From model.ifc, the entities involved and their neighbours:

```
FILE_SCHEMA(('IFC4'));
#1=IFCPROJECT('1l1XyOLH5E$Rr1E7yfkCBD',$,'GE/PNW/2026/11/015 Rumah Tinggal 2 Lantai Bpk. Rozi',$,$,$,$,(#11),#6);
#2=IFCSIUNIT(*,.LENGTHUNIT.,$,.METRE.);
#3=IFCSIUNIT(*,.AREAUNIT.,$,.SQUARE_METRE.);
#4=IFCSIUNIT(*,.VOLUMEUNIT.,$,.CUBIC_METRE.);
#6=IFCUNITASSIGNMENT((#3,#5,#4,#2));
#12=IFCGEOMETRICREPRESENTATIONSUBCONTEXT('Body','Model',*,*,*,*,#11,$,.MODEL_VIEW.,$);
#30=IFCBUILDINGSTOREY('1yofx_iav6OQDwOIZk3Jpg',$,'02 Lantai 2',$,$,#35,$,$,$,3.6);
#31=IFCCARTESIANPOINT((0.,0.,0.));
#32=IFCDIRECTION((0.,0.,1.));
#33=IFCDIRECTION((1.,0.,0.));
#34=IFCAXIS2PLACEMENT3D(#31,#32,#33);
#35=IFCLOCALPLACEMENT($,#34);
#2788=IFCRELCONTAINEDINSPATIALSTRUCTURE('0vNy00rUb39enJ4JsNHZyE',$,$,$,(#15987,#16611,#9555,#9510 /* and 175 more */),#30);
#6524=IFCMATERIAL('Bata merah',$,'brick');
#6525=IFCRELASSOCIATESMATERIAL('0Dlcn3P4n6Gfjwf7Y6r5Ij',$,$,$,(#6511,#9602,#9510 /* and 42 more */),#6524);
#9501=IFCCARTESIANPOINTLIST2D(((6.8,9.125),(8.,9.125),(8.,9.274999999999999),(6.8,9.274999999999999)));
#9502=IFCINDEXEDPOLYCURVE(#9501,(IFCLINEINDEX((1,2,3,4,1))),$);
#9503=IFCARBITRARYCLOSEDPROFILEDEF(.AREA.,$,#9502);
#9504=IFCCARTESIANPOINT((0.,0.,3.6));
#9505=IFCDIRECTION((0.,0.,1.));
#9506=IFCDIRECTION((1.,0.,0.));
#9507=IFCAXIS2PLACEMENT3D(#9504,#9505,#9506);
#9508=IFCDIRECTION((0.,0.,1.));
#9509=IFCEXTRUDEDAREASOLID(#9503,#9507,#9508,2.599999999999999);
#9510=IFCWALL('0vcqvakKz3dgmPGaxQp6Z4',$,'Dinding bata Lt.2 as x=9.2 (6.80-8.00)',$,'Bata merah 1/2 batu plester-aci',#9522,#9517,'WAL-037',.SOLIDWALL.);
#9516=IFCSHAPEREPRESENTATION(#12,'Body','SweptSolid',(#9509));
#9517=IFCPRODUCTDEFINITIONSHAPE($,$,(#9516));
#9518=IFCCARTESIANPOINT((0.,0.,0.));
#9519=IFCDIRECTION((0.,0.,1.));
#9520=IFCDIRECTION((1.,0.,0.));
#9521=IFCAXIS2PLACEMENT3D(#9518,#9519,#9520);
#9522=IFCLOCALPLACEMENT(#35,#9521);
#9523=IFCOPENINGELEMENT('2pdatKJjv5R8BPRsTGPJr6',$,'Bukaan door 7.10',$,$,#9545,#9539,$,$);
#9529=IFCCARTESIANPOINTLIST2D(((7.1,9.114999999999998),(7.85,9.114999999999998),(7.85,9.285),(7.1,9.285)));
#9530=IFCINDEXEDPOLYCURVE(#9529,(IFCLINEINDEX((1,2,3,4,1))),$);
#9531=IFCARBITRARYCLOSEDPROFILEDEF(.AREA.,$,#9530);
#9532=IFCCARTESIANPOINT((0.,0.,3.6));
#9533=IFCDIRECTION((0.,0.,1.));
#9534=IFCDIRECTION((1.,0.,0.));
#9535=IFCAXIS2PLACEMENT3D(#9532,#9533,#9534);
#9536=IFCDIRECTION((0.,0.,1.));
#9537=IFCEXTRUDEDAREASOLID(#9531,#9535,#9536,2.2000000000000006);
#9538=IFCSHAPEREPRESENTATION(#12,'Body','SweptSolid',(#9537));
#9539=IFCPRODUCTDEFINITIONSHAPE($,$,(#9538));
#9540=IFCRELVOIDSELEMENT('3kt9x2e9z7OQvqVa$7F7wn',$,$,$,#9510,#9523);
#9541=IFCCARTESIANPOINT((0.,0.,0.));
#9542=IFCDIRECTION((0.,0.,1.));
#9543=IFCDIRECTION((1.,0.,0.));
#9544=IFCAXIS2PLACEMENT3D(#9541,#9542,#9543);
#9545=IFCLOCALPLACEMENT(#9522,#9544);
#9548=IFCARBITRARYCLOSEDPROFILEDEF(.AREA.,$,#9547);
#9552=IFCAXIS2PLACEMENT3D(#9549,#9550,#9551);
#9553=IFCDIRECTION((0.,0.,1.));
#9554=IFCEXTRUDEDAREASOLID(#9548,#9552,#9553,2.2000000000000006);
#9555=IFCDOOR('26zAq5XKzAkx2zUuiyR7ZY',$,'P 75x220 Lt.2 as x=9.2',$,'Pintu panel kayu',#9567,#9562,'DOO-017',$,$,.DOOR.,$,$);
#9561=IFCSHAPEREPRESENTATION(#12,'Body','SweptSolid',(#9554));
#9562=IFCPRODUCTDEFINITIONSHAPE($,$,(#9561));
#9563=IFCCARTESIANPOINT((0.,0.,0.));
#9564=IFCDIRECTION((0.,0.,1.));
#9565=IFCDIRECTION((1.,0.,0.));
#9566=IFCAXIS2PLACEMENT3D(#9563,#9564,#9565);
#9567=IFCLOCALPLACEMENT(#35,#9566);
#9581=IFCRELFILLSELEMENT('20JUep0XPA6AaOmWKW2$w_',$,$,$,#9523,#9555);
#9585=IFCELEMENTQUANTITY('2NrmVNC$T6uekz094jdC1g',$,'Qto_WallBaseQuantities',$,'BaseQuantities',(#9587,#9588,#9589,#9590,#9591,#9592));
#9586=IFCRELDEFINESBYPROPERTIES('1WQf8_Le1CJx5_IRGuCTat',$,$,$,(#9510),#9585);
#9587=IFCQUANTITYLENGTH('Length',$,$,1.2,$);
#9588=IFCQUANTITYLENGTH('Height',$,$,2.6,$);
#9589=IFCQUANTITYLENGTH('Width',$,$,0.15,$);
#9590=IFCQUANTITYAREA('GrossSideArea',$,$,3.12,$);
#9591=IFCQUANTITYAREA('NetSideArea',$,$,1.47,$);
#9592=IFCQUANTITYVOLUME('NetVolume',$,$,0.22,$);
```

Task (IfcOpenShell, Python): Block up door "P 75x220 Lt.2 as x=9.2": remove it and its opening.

```python
import ifcopenshell
import ifcopenshell.api.feature
import ifcopenshell.api.pset
import ifcopenshell.api.root
import ifcopenshell.geom
import ifcopenshell.util.element
import ifcopenshell.util.shape
import ifcopenshell.util.unit

model = ifcopenshell.open("model.ifc")
area_scale = ifcopenshell.util.unit.calculate_unit_scale(model, "AREAUNIT")
volume_scale = ifcopenshell.util.unit.calculate_unit_scale(model, "VOLUMEUNIT")
settings = ifcopenshell.geom.settings()


def volume(element):
    """Net volume in cubic metres, openings subtracted."""
    shape = ifcopenshell.geom.create_shape(settings, element)
    return ifcopenshell.util.shape.get_volume(shape.geometry)


door = model.by_guid("26zAq5XKzAkx2zUuiyR7ZY")
opening = door.FillsVoids[0].RelatingOpeningElement
wall = opening.VoidsElements[0].RelatingBuildingElement
before = volume(wall)

ifcopenshell.api.root.remove_product(model, product=door)
ifcopenshell.api.feature.remove_feature(model, feature=opening)

after = volume(wall)
thickness = 0.15  # wall thickness in metres

# Update the wall's stored quantities.
qto = model.by_id(ifcopenshell.util.element.get_pset(wall, "Qto_WallBaseQuantities", should_inherit=False)["id"])
ifcopenshell.api.pset.edit_qto(model, qto=qto, properties={
    "NetSideArea": after / thickness / area_scale,
    "NetVolume": after / volume_scale,
})

print(f"wall volume {before:.3f} -> {after:.3f} m3")

model.write("model_v2.ifc")
```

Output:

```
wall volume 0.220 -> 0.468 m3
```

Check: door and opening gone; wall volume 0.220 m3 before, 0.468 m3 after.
